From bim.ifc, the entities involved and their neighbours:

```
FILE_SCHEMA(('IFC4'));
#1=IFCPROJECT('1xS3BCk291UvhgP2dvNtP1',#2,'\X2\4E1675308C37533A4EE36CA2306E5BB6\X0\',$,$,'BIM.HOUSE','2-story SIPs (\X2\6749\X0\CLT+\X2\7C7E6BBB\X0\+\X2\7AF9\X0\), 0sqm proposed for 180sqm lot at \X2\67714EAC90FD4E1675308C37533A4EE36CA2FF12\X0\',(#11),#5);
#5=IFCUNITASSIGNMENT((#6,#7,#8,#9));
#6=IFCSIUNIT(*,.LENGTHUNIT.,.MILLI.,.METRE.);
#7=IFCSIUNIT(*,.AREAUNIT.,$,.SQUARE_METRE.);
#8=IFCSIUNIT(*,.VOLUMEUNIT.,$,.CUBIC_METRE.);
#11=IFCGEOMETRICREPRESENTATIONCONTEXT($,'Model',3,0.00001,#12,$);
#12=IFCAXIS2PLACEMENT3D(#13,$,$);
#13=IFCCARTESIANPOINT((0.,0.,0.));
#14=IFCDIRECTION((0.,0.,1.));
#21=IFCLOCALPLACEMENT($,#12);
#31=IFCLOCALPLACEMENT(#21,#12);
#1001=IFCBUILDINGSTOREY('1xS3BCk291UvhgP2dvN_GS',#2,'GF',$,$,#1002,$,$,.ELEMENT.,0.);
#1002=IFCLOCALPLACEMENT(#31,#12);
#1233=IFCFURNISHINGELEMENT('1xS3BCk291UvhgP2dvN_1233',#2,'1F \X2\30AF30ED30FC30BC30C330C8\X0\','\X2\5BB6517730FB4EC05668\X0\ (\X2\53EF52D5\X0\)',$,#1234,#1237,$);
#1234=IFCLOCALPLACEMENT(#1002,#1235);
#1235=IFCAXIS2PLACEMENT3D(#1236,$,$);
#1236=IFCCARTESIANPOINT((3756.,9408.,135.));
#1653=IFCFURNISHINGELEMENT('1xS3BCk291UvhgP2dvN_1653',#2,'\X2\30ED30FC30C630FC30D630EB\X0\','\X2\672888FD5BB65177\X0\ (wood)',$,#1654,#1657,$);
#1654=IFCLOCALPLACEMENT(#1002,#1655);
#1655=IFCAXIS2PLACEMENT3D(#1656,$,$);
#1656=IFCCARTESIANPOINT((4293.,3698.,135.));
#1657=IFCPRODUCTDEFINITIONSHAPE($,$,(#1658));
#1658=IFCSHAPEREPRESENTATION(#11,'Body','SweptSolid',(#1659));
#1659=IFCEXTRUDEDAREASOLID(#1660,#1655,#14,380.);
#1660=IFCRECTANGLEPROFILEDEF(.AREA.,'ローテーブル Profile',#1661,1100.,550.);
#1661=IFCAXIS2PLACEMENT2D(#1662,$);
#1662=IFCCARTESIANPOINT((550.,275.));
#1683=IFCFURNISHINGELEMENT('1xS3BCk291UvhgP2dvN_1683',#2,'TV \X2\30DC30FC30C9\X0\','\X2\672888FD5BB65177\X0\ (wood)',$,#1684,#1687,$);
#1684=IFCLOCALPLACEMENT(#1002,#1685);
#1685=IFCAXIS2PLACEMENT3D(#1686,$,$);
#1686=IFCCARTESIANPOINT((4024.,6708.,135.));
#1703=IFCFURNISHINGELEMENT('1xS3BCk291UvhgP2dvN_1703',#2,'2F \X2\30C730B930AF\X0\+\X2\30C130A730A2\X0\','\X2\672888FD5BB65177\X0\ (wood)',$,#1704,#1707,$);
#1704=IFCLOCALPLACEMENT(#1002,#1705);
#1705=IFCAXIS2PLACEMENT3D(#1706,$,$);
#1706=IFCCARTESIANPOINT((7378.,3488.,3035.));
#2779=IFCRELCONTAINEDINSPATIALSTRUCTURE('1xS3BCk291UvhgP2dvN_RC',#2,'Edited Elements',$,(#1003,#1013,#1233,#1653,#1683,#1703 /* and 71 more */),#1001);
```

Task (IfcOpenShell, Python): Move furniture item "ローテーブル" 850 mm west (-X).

```python
import ifcopenshell
import ifcopenshell.api.geometry
import ifcopenshell.util.placement
import ifcopenshell.util.unit

model = ifcopenshell.open("bim.ifc")
unit_scale = ifcopenshell.util.unit.calculate_unit_scale(model)

item = model.by_guid("1xS3BCk291UvhgP2dvN_1653")
matrix = ifcopenshell.util.placement.get_local_placement(item.ObjectPlacement)
matrix[0, 3] -= 0.85 / unit_scale
ifcopenshell.api.geometry.edit_object_placement(model, product=item, matrix=matrix, is_si=False)

print(ifcopenshell.util.placement.get_local_placement(item.ObjectPlacement).round(3) + 0.0)

model.write("bim_edited.ifc")
```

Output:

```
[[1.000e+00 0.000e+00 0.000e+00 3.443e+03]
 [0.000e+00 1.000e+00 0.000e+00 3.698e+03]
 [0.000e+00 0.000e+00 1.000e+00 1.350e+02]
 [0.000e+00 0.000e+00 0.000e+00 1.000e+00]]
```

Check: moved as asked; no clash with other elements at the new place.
